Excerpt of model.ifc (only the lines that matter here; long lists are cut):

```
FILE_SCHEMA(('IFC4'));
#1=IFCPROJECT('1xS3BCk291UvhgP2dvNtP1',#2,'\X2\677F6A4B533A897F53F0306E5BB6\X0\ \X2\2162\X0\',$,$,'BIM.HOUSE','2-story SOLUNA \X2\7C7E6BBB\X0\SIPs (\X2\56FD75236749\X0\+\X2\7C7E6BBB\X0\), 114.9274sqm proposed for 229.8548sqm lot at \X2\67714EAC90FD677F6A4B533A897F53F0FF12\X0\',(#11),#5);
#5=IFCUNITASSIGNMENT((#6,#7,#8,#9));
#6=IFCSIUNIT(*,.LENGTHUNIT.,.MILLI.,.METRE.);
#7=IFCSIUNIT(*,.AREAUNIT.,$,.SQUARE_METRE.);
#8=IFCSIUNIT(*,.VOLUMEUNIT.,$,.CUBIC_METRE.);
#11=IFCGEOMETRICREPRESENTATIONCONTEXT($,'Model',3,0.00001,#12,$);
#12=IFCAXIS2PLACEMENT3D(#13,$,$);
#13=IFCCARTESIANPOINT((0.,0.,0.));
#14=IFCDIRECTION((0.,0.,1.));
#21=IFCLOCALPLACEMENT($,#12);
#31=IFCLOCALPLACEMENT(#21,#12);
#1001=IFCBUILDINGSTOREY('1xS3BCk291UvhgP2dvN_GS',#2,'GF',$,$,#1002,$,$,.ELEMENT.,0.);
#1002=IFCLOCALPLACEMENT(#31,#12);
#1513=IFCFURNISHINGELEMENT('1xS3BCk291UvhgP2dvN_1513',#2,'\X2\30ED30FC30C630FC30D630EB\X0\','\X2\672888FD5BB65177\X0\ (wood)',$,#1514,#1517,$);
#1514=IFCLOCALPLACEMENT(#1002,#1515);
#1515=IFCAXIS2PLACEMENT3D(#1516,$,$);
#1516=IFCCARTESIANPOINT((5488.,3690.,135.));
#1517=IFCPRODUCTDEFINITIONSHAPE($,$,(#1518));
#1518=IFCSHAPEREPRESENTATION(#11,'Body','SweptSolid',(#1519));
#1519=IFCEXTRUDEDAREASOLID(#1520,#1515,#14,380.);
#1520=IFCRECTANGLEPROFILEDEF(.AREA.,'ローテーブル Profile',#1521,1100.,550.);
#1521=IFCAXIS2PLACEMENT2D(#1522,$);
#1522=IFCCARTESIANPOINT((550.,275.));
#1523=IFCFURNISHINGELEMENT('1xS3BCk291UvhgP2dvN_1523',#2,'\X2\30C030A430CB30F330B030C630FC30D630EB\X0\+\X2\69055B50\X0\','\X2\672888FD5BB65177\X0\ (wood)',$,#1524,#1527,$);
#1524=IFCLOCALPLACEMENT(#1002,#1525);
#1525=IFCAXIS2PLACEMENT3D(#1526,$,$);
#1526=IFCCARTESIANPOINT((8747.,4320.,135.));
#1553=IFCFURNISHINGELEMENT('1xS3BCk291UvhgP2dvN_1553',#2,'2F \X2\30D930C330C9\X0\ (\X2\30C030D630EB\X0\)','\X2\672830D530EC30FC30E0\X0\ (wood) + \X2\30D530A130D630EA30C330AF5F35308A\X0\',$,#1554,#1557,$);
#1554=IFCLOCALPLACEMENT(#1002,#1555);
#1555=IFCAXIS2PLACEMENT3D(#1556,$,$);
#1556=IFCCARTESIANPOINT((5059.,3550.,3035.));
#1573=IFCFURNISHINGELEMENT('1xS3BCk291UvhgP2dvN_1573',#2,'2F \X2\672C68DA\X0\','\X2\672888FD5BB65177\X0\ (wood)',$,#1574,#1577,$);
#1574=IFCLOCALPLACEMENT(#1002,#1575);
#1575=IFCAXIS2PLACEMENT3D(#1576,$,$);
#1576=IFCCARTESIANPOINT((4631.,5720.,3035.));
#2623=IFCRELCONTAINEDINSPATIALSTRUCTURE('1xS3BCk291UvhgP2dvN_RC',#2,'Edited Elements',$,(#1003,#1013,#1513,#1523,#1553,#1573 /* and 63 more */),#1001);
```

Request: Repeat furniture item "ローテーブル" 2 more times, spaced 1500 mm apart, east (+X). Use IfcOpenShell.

```python
import numpy as np
import ifcopenshell
import ifcopenshell.api.geometry
import ifcopenshell.api.root
import ifcopenshell.util.element
import ifcopenshell.util.placement
import ifcopenshell.util.unit

model = ifcopenshell.open("model.ifc")
unit_scale = ifcopenshell.util.unit.calculate_unit_scale(model)


def reuse_history(source, copy):
    """copy_class also copies each property set's owner history, people and application; keep the originals."""
    for rel in copy.IsDefinedBy:
        if rel.is_a("IfcRelDefinesByProperties") and (history := rel.RelatingPropertyDefinition.OwnerHistory):
            rel.RelatingPropertyDefinition.OwnerHistory = source.OwnerHistory
            ifcopenshell.util.element.remove_deep2(model, history)


source = model.by_guid("1xS3BCk291UvhgP2dvN_1513")
base = ifcopenshell.util.placement.get_local_placement(source.ObjectPlacement)
step = np.array([1.0, 0.0, 0.0]) * 1.5 / unit_scale

for i in range(1, 3):
    copy = ifcopenshell.api.root.copy_class(model, product=source)
    copy.Representation = ifcopenshell.util.element.copy_deep(
        model, source.Representation, exclude=["IfcGeometricRepresentationContext", "IfcRepresentationMap"]
    )
    reuse_history(source, copy)
    matrix = base.copy()
    matrix[:3, 3] += i * step
    print("added at", matrix[:3, 3].round(3) + 0.0)
    ifcopenshell.api.geometry.edit_object_placement(model, product=copy, matrix=matrix, is_si=False)

model.write("model_rev.ifc")
```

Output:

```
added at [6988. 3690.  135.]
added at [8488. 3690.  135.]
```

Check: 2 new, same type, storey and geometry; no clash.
